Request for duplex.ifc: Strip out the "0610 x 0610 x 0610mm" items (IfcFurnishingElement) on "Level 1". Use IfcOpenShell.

First a look at what the model holds.

```python
import ifcopenshell
import ifcopenshell.util.element

model = ifcopenshell.open("duplex.ifc")
print(model.schema)
storey = next(s for s in model.by_type("IfcBuildingStorey") if s.Name == "Level 1")
furniture = [e for e in ifcopenshell.util.element.get_decomposition(storey) if e.is_a("IfcFurnishingElement")]
seen = {}
for e in furniture:
    element_type = ifcopenshell.util.element.get_type(e)
    name = element_type.Name if element_type not in (None, e) else None
    seen[name] = seen.get(name, 0) + 1
for name, count in sorted(seen.items(), key=str):
    print(count, "x", name)
```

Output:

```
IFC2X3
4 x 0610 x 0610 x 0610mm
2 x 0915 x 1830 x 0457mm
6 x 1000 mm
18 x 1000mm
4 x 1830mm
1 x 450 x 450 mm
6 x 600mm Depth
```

```python
import ifcopenshell
import ifcopenshell.api.root
import ifcopenshell.util.element

model = ifcopenshell.open("duplex.ifc")

storey = next(s for s in model.by_type("IfcBuildingStorey") if s.Name == "Level 1")
furniture = [e for e in ifcopenshell.util.element.get_decomposition(storey) if e.is_a("IfcFurnishingElement")]
targets = [e for e in furniture if (t := ifcopenshell.util.element.get_type(e)) not in (None, e) and t.Name == "0610 x 0610 x 0610mm"]

for e in targets:
    ifcopenshell.api.root.remove_product(model, product=e)
print(len(targets), "removed")

model.write("duplex_v2.ifc")
```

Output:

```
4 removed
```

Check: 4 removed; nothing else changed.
